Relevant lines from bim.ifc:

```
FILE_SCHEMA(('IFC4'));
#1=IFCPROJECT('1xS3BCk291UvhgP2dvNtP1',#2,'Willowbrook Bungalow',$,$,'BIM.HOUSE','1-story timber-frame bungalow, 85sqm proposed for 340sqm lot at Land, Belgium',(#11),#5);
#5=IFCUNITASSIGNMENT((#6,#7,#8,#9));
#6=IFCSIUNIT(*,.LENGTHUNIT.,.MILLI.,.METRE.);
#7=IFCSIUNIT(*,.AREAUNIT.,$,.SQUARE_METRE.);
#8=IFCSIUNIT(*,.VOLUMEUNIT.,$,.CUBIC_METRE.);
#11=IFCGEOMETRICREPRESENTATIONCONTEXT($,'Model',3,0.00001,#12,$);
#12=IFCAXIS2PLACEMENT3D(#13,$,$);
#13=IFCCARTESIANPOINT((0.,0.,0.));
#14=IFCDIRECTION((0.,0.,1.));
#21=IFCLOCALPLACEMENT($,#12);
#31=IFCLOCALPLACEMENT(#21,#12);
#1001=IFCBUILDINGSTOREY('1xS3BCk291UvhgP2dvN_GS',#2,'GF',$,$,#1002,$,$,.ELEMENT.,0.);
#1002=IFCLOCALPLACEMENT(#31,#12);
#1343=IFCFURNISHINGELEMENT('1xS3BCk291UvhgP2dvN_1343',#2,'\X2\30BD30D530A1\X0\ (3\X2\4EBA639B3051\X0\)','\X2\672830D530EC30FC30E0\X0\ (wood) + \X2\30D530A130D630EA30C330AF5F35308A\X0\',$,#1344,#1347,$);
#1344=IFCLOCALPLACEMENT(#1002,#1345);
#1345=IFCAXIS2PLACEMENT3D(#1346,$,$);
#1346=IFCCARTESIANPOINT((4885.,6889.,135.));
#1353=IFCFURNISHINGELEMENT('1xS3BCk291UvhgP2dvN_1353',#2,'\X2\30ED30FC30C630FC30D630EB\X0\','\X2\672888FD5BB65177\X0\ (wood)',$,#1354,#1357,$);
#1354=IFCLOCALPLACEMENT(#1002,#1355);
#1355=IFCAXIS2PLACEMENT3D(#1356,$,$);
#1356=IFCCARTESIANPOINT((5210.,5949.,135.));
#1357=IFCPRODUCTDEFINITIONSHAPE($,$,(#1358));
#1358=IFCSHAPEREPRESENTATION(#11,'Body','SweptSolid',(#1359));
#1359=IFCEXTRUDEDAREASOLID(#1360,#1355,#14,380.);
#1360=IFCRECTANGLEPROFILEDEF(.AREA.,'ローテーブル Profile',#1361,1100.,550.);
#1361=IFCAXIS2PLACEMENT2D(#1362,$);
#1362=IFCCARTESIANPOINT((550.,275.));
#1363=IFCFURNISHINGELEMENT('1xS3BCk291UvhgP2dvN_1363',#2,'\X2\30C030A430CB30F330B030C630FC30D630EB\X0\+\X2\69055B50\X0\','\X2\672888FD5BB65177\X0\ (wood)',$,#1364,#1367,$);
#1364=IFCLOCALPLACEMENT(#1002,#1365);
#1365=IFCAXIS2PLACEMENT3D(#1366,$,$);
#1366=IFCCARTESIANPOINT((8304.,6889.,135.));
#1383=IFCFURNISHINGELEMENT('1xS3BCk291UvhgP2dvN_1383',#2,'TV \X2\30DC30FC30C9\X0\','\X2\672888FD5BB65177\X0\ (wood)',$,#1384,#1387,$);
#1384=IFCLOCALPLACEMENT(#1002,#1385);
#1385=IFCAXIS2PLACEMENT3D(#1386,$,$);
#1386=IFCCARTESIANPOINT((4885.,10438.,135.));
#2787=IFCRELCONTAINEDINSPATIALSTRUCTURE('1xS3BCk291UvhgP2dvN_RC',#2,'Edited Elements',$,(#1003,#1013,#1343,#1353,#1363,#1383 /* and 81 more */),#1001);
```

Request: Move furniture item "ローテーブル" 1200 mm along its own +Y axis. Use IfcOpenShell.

```python
import ifcopenshell
import ifcopenshell.api.geometry
import ifcopenshell.util.placement
import ifcopenshell.util.unit

model = ifcopenshell.open("bim.ifc")
unit_scale = ifcopenshell.util.unit.calculate_unit_scale(model)

item = model.by_guid("1xS3BCk291UvhgP2dvN_1353")
matrix = ifcopenshell.util.placement.get_local_placement(item.ObjectPlacement)
matrix[:3, 3] += matrix[:3, 1] * 1.2 / unit_scale
ifcopenshell.api.geometry.edit_object_placement(model, product=item, matrix=matrix, is_si=False)

print(ifcopenshell.util.placement.get_local_placement(item.ObjectPlacement).round(3) + 0.0)

model.write("bim_v2.ifc")
```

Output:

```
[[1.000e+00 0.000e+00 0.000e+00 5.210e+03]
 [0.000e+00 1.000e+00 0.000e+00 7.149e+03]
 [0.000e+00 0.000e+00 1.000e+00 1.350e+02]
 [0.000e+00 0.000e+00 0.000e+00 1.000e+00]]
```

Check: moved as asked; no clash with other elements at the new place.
